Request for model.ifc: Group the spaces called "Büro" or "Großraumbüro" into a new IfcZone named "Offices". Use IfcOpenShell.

First a look at what the model holds.

```python
import ifcopenshell

model = ifcopenshell.open("model.ifc")
print(model.schema)
seen = {}
for space in model.by_type("IfcSpace"):
    seen[space.LongName] = seen.get(space.LongName, 0) + 1
for name, count in sorted(seen.items(), key=str):
    print(count, "x", name)
print("zones:", [z.Name for z in model.by_type("IfcZone")][:20])
```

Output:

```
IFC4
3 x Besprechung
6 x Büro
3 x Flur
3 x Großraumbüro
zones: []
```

```python
import ifcopenshell
import ifcopenshell.api.group
import ifcopenshell.api.root

model = ifcopenshell.open("model.ifc")

names = {"Büro", "Großraumbüro"}
spaces = [s for s in model.by_type("IfcSpace") if s.LongName in names]

zone = ifcopenshell.api.root.create_entity(model, ifc_class="IfcZone", name="Offices")
ifcopenshell.api.group.assign_group(model, products=spaces, group=zone)
print(len(spaces), "spaces in", zone.Name)

model.write("model_updated.ifc")
```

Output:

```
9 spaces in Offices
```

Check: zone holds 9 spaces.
